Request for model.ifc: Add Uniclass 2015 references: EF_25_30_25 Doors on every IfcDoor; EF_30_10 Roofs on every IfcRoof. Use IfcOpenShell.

First a look at what the model holds.

```python
import ifcopenshell

model = ifcopenshell.open("model.ifc")
print(model.schema)
print("classifications:", [c.Name for c in model.by_type("IfcClassification")])
for ifc_class in ("IfcDoor", "IfcRoof", "IfcStair", "IfcWall", "IfcWindow"):
    print(ifc_class, len(model.by_type(ifc_class)))
```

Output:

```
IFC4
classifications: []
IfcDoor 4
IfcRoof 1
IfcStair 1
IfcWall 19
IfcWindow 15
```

```python
import ifcopenshell
import ifcopenshell.api.classification

model = ifcopenshell.open("model.ifc")

system = ifcopenshell.api.classification.add_classification(model, classification="Uniclass 2015")

codes = {
    "IfcDoor": ("EF_25_30_25", "Doors"),
    "IfcRoof": ("EF_30_10", "Roofs"),
}
for ifc_class, (code, name) in codes.items():
    products = model.by_type(ifc_class)
    ifcopenshell.api.classification.add_reference(
        model, products=products, classification=system, identification=code, name=name
    )
    print(code, len(products))

model.write("model_v2.ifc")
```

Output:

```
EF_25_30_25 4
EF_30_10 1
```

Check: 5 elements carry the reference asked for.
